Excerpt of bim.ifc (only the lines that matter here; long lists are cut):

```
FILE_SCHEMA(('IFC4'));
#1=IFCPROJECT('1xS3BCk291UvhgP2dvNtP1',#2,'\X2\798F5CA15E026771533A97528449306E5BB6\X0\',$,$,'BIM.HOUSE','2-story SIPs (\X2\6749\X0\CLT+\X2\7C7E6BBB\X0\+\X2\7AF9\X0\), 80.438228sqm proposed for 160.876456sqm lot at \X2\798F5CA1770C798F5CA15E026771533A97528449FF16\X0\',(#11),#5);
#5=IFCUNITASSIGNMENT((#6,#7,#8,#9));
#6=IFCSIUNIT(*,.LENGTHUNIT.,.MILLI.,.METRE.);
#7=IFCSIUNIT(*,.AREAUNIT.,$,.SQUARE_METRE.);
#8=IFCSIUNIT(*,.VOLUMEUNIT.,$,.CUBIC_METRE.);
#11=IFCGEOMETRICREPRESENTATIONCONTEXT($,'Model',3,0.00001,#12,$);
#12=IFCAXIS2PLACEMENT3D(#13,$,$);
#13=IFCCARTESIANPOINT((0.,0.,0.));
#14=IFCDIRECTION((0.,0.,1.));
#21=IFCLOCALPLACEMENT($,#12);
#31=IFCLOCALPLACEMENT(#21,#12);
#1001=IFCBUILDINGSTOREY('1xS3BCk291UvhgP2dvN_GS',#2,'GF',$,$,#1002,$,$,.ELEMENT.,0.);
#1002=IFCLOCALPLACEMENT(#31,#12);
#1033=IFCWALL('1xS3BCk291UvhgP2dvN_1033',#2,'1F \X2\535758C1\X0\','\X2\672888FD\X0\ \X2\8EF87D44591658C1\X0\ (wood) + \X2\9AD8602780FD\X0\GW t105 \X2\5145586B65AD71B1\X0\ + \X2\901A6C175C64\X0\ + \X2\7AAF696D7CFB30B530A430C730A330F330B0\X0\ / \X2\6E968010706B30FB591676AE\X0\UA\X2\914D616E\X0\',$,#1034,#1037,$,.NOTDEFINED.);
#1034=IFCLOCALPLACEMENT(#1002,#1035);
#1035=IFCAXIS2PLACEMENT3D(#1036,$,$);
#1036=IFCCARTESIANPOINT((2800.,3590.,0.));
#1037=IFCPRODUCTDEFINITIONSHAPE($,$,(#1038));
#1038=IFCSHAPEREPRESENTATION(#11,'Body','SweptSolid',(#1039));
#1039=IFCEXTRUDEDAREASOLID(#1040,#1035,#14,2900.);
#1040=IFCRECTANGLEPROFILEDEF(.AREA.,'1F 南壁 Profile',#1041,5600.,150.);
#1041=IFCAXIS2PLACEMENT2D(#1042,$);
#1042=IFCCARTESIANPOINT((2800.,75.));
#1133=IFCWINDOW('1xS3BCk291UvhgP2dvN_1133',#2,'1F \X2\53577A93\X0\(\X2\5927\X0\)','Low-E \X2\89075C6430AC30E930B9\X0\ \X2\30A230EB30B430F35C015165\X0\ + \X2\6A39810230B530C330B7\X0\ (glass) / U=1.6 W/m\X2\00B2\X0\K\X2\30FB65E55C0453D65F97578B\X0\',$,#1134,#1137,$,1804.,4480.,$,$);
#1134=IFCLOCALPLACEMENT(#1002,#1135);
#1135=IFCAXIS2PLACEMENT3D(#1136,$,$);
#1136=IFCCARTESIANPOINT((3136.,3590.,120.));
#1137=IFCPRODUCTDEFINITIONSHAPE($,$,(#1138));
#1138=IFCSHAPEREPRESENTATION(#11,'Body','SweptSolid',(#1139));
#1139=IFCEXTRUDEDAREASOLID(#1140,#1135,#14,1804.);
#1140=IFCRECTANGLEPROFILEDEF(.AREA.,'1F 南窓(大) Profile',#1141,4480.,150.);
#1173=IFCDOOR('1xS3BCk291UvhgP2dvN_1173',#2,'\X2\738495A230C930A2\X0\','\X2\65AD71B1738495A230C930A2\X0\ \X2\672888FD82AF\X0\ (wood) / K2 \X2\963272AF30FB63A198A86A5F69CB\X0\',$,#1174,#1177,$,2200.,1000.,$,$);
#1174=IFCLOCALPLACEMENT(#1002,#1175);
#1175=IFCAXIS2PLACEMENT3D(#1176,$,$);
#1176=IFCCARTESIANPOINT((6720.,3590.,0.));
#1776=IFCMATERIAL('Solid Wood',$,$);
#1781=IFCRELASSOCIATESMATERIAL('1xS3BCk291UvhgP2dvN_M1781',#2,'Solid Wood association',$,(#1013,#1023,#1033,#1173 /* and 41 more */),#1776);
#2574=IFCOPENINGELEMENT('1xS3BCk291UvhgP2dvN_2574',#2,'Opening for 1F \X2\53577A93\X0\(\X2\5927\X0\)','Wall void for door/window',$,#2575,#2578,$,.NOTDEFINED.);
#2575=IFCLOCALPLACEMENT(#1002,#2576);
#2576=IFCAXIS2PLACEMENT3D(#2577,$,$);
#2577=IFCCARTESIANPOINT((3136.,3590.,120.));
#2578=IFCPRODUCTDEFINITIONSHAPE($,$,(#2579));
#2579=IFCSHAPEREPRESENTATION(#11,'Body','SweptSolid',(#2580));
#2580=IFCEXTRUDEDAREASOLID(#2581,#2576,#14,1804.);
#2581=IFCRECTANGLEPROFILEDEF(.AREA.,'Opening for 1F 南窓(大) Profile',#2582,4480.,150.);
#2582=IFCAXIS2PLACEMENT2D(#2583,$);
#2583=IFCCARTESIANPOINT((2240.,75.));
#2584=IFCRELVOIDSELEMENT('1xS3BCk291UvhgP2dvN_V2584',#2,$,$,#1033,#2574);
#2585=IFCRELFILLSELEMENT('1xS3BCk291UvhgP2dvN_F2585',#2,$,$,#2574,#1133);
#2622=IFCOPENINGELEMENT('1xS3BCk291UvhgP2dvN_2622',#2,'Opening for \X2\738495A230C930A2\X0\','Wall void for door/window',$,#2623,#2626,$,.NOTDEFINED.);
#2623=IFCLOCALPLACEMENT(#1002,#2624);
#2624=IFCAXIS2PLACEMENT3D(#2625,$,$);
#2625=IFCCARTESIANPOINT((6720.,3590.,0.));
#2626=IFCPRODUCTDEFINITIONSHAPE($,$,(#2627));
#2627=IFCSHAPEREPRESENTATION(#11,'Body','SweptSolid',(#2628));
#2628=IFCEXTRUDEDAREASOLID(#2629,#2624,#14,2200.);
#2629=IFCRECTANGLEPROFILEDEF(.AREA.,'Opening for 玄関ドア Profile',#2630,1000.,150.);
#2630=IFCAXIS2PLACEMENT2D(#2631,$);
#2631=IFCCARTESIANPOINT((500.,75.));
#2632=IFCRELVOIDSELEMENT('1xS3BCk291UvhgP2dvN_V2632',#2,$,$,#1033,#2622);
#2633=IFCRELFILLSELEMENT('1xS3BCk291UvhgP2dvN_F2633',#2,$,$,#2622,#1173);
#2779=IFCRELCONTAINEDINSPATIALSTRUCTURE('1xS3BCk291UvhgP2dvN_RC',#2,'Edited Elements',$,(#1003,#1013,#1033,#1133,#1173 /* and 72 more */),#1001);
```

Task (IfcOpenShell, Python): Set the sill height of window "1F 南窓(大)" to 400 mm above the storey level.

```python
import numpy as np
import ifcopenshell
import ifcopenshell.api.geometry
import ifcopenshell.geom
import ifcopenshell.util.element
import ifcopenshell.util.placement
import ifcopenshell.util.shape
import ifcopenshell.util.unit

model = ifcopenshell.open("bim.ifc")
unit_scale = ifcopenshell.util.unit.calculate_unit_scale(model)

window = model.by_guid("1xS3BCk291UvhgP2dvN_1133")
opening = window.FillsVoids[0].RelatingOpeningElement
storey = ifcopenshell.util.element.get_container(window, ifc_class="IfcBuildingStorey")
level = ifcopenshell.util.placement.get_local_placement(storey.ObjectPlacement)[2, 3]

# The opening's origin need not be at the sill, so measure its lowest point.
shape = ifcopenshell.geom.create_shape(ifcopenshell.geom.settings(), opening)
bottom = ifcopenshell.util.shape.get_shape_bottom_elevation(shape, shape.geometry) / unit_scale
dz = level + 0.4 / unit_scale - bottom

shift = np.array([0.0, 0.0, dz])
# The window is not placed relative to its opening, so move both.
for product in (opening, window):
    matrix = ifcopenshell.util.placement.get_local_placement(product.ObjectPlacement)
    matrix[:3, 3] += shift
    ifcopenshell.api.geometry.edit_object_placement(model, product=product, matrix=matrix, is_si=False)

print(f"moved by {dz * unit_scale:+.3f} m")

model.write("bim_updated.ifc")
```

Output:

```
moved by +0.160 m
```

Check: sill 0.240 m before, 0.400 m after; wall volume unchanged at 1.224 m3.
